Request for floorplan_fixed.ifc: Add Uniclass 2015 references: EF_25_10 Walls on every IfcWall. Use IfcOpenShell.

First a look at what the model holds.

```python
import ifcopenshell

model = ifcopenshell.open("floorplan_fixed.ifc")
print(model.schema)
print("classifications:", [c.Name for c in model.by_type("IfcClassification")])
for ifc_class in ("IfcDoor", "IfcRoof", "IfcStair", "IfcWall", "IfcWindow"):
    print(ifc_class, len(model.by_type(ifc_class)))
```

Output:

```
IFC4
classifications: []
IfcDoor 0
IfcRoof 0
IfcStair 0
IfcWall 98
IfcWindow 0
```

```python
import ifcopenshell
import ifcopenshell.api.classification

model = ifcopenshell.open("floorplan_fixed.ifc")

system = ifcopenshell.api.classification.add_classification(model, classification="Uniclass 2015")

codes = {
    "IfcWall": ("EF_25_10", "Walls"),
}
for ifc_class, (code, name) in codes.items():
    products = model.by_type(ifc_class)
    ifcopenshell.api.classification.add_reference(
        model, products=products, classification=system, identification=code, name=name
    )
    print(code, len(products))

model.write("floorplan_fixed_updated.ifc")
```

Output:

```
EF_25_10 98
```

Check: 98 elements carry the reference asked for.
